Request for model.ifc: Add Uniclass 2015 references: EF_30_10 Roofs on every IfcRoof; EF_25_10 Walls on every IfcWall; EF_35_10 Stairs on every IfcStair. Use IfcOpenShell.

First a look at what the model holds.

```python
import ifcopenshell

model = ifcopenshell.open("model.ifc")
print(model.schema)
print("classifications:", [c.Name for c in model.by_type("IfcClassification")])
for ifc_class in ("IfcDoor", "IfcRoof", "IfcStair", "IfcWall", "IfcWindow"):
    print(ifc_class, len(model.by_type(ifc_class)))
```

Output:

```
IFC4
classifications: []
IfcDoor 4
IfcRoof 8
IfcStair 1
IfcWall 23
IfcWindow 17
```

```python
import ifcopenshell
import ifcopenshell.api.classification

model = ifcopenshell.open("model.ifc")

system = ifcopenshell.api.classification.add_classification(model, classification="Uniclass 2015")

codes = {
    "IfcRoof": ("EF_30_10", "Roofs"),
    "IfcWall": ("EF_25_10", "Walls"),
    "IfcStair": ("EF_35_10", "Stairs"),
}
for ifc_class, (code, name) in codes.items():
    products = model.by_type(ifc_class)
    ifcopenshell.api.classification.add_reference(
        model, products=products, classification=system, identification=code, name=name
    )
    print(code, len(products))

model.write("model_updated.ifc")
```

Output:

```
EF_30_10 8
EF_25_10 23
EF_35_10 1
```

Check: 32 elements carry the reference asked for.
